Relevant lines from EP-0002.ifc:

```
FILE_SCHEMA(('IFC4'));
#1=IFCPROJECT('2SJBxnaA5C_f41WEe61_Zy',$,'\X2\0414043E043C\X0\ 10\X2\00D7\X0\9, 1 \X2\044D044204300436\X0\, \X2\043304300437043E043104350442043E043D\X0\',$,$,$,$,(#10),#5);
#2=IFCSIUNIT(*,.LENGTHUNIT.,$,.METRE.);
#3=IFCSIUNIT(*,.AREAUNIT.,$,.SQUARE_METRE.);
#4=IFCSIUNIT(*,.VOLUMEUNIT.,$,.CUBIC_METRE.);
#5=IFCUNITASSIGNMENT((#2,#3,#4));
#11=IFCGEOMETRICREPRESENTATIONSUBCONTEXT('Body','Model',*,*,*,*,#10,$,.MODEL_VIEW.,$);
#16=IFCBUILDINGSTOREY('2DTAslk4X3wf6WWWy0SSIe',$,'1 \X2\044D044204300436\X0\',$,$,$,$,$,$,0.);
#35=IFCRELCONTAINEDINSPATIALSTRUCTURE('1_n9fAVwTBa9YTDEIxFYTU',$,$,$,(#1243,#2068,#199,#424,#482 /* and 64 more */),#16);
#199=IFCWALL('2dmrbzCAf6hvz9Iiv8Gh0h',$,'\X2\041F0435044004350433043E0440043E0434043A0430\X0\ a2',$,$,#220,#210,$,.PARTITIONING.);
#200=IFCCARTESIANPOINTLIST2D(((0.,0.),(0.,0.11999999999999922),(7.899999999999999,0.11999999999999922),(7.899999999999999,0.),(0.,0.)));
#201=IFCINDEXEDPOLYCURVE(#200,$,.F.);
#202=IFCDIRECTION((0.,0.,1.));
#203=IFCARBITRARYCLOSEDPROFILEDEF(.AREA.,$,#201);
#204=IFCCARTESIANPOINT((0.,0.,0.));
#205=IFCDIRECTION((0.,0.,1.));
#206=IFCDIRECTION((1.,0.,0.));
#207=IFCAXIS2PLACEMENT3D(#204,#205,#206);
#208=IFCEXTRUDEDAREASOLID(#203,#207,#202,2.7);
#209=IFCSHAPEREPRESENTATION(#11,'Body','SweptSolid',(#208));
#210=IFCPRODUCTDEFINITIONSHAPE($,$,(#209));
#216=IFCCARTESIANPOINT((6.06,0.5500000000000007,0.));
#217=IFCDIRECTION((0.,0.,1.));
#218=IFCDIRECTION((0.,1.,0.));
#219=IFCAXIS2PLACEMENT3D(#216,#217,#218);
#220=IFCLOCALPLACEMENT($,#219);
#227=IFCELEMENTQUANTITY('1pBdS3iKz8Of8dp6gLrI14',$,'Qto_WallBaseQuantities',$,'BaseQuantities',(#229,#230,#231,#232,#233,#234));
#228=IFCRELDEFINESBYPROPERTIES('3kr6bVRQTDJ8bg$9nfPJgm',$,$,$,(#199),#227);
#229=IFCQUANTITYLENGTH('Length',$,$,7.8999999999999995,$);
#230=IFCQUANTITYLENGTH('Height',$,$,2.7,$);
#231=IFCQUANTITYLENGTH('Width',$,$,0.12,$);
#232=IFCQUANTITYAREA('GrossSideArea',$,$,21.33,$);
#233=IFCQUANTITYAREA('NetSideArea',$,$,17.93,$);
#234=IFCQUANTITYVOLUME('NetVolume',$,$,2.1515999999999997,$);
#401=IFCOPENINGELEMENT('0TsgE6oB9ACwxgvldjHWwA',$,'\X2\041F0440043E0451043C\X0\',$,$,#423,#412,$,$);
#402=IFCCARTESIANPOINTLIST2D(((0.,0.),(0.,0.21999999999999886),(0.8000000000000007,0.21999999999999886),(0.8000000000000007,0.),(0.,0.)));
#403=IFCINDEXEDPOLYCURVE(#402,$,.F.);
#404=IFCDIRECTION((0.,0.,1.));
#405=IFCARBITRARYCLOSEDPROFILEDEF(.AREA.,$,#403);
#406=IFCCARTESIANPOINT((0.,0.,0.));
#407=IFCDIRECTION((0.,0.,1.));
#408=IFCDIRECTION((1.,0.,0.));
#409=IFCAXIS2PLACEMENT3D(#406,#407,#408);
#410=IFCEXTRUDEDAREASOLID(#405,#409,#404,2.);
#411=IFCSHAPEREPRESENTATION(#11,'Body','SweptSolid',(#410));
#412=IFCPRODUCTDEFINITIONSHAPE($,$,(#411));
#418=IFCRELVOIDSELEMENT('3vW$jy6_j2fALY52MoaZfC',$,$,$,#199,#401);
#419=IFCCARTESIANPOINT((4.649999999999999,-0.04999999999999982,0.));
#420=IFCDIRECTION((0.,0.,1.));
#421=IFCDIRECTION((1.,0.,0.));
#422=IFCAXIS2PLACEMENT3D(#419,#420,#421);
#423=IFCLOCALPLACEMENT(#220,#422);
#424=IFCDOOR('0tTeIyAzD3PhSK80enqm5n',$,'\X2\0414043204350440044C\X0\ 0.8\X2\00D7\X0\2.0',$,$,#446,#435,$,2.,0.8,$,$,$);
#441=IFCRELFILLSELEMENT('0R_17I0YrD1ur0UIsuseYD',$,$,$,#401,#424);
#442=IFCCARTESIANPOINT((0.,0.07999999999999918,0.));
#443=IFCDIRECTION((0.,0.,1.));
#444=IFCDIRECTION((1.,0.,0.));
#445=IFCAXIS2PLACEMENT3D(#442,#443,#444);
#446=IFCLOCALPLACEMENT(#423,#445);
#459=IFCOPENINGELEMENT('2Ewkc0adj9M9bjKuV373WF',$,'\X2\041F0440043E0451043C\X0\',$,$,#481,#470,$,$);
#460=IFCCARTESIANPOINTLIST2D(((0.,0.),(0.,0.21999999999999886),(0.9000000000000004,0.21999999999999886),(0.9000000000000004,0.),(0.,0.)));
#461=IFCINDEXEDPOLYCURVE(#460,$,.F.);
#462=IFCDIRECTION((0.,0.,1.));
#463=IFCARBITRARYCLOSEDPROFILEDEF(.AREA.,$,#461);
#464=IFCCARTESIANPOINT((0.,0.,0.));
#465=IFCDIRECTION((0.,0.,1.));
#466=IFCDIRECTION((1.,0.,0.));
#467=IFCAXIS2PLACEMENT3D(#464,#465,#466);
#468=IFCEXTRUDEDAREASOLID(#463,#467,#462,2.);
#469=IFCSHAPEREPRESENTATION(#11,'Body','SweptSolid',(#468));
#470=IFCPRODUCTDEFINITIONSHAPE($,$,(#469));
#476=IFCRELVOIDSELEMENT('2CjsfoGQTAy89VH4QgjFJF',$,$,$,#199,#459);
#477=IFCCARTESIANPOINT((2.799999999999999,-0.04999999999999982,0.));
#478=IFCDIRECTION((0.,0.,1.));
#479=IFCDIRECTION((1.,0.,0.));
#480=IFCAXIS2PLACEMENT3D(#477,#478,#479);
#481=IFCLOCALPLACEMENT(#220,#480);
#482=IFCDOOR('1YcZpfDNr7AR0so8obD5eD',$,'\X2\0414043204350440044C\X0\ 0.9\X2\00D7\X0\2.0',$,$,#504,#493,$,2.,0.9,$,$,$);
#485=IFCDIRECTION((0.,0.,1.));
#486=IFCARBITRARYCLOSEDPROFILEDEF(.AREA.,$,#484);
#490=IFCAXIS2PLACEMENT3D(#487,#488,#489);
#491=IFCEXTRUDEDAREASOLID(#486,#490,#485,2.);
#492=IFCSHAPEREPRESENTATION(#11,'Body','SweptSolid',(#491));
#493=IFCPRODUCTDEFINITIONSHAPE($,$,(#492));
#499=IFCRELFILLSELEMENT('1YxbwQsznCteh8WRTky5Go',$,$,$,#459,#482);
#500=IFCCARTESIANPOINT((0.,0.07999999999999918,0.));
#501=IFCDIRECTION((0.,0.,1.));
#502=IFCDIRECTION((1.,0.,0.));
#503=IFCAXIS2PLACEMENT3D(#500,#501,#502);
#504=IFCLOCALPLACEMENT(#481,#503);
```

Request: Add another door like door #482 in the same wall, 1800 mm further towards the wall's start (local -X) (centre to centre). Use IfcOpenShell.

```python
import ifcopenshell
import ifcopenshell.api.feature
import ifcopenshell.api.geometry
import ifcopenshell.api.pset
import ifcopenshell.api.root
import ifcopenshell.geom
import ifcopenshell.util.element
import ifcopenshell.util.placement
import ifcopenshell.util.shape
import ifcopenshell.util.unit

model = ifcopenshell.open("EP-0002.ifc")
unit_scale = ifcopenshell.util.unit.calculate_unit_scale(model)
area_scale = ifcopenshell.util.unit.calculate_unit_scale(model, "AREAUNIT")
volume_scale = ifcopenshell.util.unit.calculate_unit_scale(model, "VOLUMEUNIT")
settings = ifcopenshell.geom.settings()


def volume(element):
    """Net volume in cubic metres, openings subtracted."""
    shape = ifcopenshell.geom.create_shape(settings, element)
    return ifcopenshell.util.shape.get_volume(shape.geometry)


door = model.by_guid("1YcZpfDNr7AR0so8obD5eD")
opening = door.FillsVoids[0].RelatingOpeningElement
wall = opening.VoidsElements[0].RelatingBuildingElement
before = volume(wall)
shift = ifcopenshell.util.placement.get_local_placement(wall.ObjectPlacement)[:3, 0] * -1.8 / unit_scale

# copy_class copies the void relationship, type, container and properties, but no geometry.
new_opening = ifcopenshell.api.root.copy_class(model, product=opening)
new_opening.Representation = ifcopenshell.util.element.copy_deep(
    model, opening.Representation, exclude=["IfcGeometricRepresentationContext", "IfcRepresentationMap"]
)
new_door = ifcopenshell.api.root.copy_class(model, product=door)
new_door.Representation = ifcopenshell.util.element.copy_deep(
    model, door.Representation, exclude=["IfcGeometricRepresentationContext", "IfcRepresentationMap"]
)
ifcopenshell.api.feature.add_filling(model, opening=new_opening, element=new_door)

for old, new in ((opening, new_opening), (door, new_door)):
    matrix = ifcopenshell.util.placement.get_local_placement(old.ObjectPlacement)
    matrix[:3, 3] += shift
    ifcopenshell.api.geometry.edit_object_placement(model, product=new, matrix=matrix, is_si=False)

after = volume(wall)
thickness = 0.12  # wall thickness in metres

# Update the wall's stored quantities.
qto = model.by_id(ifcopenshell.util.element.get_pset(wall, "Qto_WallBaseQuantities", should_inherit=False)["id"])
ifcopenshell.api.pset.edit_qto(model, qto=qto, properties={
    "NetSideArea": after / thickness / area_scale,
    "NetVolume": after / volume_scale,
})

print(f"wall volume {before:.3f} -> {after:.3f} m3")

model.write("EP-0002_rev.ifc")
```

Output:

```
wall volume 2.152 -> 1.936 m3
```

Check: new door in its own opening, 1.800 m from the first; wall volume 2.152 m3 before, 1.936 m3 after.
